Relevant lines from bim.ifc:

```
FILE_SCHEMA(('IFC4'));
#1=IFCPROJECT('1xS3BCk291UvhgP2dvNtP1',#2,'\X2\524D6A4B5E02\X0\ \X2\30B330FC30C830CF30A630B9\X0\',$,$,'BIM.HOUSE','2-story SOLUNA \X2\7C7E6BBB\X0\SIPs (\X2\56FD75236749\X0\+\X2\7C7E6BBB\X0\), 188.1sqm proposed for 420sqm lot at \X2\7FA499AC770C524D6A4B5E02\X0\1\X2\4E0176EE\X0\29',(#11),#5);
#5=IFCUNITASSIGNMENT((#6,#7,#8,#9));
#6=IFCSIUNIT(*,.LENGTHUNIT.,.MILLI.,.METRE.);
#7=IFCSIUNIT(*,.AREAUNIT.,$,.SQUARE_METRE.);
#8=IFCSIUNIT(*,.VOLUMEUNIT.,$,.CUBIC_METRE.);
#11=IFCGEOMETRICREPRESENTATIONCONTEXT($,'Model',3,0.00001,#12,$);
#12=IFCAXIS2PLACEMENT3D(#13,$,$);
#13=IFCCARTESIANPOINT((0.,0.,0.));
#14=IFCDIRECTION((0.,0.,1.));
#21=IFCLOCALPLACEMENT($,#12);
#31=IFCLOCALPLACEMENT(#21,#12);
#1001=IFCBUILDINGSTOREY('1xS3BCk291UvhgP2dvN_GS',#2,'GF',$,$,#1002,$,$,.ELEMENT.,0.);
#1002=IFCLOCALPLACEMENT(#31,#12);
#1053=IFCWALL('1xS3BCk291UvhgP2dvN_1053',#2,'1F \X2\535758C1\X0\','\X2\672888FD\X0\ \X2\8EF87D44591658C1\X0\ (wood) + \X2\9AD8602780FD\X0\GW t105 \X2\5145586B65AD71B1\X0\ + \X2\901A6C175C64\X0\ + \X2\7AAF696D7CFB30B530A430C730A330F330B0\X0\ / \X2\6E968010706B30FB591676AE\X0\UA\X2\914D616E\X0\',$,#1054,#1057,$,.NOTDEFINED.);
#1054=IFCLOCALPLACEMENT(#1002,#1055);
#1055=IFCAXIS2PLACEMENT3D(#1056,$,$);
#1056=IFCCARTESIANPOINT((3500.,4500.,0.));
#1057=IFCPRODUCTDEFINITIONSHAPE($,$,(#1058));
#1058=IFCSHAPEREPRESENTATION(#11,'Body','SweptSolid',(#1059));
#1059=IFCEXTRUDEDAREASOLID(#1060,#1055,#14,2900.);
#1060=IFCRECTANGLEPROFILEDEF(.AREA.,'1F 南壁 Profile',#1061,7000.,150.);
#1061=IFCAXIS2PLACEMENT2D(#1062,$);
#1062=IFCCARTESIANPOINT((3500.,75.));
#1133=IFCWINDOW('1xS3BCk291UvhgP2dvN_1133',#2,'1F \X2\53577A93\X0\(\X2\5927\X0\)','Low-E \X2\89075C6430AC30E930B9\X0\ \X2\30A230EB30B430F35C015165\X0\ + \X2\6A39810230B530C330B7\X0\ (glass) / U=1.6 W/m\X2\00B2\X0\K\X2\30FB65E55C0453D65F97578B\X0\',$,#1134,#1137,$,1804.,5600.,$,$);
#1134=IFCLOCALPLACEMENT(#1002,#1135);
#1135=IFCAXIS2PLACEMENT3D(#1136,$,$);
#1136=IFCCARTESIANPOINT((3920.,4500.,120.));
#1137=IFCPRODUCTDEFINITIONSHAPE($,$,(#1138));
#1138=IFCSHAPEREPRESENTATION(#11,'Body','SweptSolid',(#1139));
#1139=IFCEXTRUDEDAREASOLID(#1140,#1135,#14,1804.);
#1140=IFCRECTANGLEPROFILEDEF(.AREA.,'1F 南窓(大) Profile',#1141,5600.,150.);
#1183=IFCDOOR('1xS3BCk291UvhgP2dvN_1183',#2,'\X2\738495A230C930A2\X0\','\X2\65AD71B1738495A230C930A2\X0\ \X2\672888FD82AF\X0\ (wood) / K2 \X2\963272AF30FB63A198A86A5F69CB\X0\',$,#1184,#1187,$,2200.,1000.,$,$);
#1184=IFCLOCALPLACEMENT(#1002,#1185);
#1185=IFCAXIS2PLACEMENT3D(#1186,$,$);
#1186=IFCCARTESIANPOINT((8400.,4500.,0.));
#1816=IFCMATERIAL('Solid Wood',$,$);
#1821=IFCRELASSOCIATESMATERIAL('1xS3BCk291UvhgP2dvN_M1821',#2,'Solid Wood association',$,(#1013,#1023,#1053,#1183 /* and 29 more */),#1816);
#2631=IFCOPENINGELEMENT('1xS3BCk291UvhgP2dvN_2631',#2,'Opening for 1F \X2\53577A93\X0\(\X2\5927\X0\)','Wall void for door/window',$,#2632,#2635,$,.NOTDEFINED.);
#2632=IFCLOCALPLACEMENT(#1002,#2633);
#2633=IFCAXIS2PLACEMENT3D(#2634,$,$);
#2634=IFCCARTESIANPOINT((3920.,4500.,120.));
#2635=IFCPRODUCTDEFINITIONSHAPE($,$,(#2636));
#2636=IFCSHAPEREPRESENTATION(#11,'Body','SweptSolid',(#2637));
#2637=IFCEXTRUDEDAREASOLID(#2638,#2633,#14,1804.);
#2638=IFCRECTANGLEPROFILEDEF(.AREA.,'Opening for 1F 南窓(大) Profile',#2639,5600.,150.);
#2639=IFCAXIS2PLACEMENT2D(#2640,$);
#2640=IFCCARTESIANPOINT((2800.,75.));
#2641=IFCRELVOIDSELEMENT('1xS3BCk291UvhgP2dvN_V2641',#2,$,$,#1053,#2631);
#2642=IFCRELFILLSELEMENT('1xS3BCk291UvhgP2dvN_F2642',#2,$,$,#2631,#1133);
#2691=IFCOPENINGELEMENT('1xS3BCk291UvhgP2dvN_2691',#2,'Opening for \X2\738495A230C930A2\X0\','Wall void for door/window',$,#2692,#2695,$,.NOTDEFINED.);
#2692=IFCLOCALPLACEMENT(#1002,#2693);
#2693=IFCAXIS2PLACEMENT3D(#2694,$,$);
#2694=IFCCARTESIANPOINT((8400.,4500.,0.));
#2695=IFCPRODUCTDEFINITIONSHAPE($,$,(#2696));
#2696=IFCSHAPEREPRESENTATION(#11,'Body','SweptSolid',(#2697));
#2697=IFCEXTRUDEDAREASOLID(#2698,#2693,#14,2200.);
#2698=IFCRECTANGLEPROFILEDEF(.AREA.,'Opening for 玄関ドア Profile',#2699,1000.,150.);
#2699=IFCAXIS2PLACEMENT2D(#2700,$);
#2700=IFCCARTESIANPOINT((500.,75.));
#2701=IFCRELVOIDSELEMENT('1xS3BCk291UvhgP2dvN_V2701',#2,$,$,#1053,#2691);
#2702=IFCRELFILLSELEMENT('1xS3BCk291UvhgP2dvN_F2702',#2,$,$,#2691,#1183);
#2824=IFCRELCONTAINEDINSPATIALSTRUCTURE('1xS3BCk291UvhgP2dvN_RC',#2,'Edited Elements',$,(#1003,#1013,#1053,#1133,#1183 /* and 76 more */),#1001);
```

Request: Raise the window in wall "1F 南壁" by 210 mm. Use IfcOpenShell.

```python
import numpy as np
import ifcopenshell
import ifcopenshell.api.geometry
import ifcopenshell.util.placement
import ifcopenshell.util.unit

model = ifcopenshell.open("bim.ifc")
unit_scale = ifcopenshell.util.unit.calculate_unit_scale(model)

window = model.by_id(1133)
opening = window.FillsVoids[0].RelatingOpeningElement
dz = 210.0

shift = np.array([0.0, 0.0, dz])
# The window is not placed relative to its opening, so move both.
for product in (opening, window):
    matrix = ifcopenshell.util.placement.get_local_placement(product.ObjectPlacement)
    matrix[:3, 3] += shift
    ifcopenshell.api.geometry.edit_object_placement(model, product=product, matrix=matrix, is_si=False)

print(f"moved by {dz * unit_scale:+.3f} m")

model.write("bim_edited.ifc")
```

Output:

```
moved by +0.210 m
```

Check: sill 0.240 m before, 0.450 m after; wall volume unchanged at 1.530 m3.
